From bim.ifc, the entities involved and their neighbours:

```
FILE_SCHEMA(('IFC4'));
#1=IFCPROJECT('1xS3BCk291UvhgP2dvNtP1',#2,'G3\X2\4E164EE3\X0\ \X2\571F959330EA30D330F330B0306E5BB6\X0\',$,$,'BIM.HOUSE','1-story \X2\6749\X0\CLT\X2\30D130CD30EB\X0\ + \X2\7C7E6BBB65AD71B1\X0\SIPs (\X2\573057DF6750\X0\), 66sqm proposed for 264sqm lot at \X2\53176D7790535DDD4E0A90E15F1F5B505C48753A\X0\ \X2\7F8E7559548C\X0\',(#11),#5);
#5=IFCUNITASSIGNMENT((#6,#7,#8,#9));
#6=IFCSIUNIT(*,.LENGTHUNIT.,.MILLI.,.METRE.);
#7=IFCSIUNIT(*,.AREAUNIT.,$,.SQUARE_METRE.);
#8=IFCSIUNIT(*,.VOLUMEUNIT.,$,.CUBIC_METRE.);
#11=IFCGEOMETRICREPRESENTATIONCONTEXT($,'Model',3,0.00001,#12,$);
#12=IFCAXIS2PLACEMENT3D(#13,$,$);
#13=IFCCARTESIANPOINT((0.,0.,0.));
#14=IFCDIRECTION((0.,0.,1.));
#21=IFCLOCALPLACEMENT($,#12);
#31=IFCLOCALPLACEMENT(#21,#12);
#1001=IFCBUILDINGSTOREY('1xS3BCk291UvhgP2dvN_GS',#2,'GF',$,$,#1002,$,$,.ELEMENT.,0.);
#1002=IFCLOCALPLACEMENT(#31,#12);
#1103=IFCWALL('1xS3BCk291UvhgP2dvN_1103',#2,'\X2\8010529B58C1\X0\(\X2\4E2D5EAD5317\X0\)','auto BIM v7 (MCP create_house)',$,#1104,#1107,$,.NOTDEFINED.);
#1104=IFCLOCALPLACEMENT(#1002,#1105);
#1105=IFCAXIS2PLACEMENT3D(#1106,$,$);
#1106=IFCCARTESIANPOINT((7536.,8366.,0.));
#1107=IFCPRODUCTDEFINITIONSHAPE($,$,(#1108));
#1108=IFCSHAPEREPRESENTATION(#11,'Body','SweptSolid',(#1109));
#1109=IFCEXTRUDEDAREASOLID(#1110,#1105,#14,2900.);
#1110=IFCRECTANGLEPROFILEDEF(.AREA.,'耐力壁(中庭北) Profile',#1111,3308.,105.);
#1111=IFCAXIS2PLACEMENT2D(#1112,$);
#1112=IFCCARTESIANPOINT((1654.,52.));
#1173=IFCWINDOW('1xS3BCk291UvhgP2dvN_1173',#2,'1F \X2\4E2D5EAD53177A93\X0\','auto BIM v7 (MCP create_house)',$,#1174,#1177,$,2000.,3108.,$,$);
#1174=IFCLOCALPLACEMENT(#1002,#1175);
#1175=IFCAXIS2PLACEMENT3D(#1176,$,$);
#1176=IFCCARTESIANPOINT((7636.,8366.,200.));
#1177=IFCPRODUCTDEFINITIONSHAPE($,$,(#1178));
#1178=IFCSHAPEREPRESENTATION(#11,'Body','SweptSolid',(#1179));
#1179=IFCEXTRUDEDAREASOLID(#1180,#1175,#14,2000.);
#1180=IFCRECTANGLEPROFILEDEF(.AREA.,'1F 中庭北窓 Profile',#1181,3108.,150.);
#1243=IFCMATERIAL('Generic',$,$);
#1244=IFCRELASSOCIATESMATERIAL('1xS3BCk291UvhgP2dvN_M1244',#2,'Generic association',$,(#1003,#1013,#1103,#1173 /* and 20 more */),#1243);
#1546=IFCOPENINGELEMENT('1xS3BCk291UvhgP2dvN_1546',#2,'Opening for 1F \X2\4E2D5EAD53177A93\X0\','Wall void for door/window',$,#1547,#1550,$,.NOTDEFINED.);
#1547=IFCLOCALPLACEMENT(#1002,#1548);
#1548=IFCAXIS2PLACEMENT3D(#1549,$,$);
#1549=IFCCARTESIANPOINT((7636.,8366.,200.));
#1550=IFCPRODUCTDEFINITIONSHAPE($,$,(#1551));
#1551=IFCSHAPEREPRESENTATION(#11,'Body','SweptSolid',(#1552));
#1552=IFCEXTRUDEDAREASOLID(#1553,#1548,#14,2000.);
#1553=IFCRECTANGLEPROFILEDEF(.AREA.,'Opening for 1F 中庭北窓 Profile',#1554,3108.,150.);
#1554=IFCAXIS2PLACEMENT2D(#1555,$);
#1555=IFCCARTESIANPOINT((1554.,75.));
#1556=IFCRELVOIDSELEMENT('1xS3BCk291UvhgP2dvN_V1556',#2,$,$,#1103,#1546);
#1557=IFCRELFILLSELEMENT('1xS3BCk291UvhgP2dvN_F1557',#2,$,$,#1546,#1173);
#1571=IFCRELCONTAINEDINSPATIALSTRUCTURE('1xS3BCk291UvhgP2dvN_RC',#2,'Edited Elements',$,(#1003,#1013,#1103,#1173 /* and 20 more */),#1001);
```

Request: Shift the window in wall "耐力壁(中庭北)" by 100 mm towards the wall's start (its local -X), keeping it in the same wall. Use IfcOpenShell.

```python
import ifcopenshell
import ifcopenshell.api.geometry
import ifcopenshell.util.placement
import ifcopenshell.util.unit

model = ifcopenshell.open("bim.ifc")
unit_scale = ifcopenshell.util.unit.calculate_unit_scale(model)

window = model.by_guid("1xS3BCk291UvhgP2dvN_1173")
opening = window.FillsVoids[0].RelatingOpeningElement
wall = opening.VoidsElements[0].RelatingBuildingElement

wall_matrix = ifcopenshell.util.placement.get_local_placement(wall.ObjectPlacement)
shift = wall_matrix[:3, 0] * -0.1 / unit_scale
before = ifcopenshell.util.placement.get_local_placement(window.ObjectPlacement)[:3, 3].copy()

# The window is not placed relative to its opening, so move both.
for product in (opening, window):
    matrix = ifcopenshell.util.placement.get_local_placement(product.ObjectPlacement)
    matrix[:3, 3] += shift
    ifcopenshell.api.geometry.edit_object_placement(model, product=product, matrix=matrix, is_si=False)

after = ifcopenshell.util.placement.get_local_placement(window.ObjectPlacement)[:3, 3]
print("window moved by", (after - before).round(3) + 0.0)

model.write("bim_rev.ifc")
```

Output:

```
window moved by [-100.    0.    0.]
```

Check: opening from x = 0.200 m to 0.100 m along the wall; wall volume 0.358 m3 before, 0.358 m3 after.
